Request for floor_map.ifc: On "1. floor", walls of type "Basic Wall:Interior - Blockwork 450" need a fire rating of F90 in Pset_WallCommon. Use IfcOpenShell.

First a look at what the model holds.

```python
import ifcopenshell
import ifcopenshell.util.element

model = ifcopenshell.open("floor_map.ifc")
print(model.schema)
storey = next(s for s in model.by_type("IfcBuildingStorey") if s.Name == "1. floor")
walls = [e for e in ifcopenshell.util.element.get_decomposition(storey) if e.is_a("IfcWall")]
seen = {}
for e in walls:
    element_type = ifcopenshell.util.element.get_type(e)
    key = (element_type.Name if element_type != e and element_type else None, ifcopenshell.util.element.get_pset(e, "Pset_WallCommon", "FireRating"))
    seen[key] = seen.get(key, 0) + 1
for (name, value), count in sorted(seen.items(), key=str):
    print(count, "x", name, "|", value)
```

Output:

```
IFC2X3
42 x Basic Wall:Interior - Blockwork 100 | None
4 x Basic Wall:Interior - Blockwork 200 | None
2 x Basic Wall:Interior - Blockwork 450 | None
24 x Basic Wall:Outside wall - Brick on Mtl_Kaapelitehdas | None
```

```python
import ifcopenshell
import ifcopenshell.api.pset
import ifcopenshell.util.element

model = ifcopenshell.open("floor_map.ifc")

storey = next(s for s in model.by_type("IfcBuildingStorey") if s.Name == "1. floor")
walls = [e for e in ifcopenshell.util.element.get_decomposition(storey) if e.is_a("IfcWall")]

count = 0
for e in walls:
    element_type = ifcopenshell.util.element.get_type(e)
    if element_type in (None, e) or element_type.Name != "Basic Wall:Interior - Blockwork 450":
        continue
    # add_pset returns the element's existing set when there is one.
    pset = ifcopenshell.api.pset.add_pset(model, product=e, name="Pset_WallCommon")
    ifcopenshell.api.pset.edit_pset(model, pset=pset, properties={"FireRating": "F90"})
    count += 1

print(count, "walls updated")

model.write("floor_map_rev.ifc")
```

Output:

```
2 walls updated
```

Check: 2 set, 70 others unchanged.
